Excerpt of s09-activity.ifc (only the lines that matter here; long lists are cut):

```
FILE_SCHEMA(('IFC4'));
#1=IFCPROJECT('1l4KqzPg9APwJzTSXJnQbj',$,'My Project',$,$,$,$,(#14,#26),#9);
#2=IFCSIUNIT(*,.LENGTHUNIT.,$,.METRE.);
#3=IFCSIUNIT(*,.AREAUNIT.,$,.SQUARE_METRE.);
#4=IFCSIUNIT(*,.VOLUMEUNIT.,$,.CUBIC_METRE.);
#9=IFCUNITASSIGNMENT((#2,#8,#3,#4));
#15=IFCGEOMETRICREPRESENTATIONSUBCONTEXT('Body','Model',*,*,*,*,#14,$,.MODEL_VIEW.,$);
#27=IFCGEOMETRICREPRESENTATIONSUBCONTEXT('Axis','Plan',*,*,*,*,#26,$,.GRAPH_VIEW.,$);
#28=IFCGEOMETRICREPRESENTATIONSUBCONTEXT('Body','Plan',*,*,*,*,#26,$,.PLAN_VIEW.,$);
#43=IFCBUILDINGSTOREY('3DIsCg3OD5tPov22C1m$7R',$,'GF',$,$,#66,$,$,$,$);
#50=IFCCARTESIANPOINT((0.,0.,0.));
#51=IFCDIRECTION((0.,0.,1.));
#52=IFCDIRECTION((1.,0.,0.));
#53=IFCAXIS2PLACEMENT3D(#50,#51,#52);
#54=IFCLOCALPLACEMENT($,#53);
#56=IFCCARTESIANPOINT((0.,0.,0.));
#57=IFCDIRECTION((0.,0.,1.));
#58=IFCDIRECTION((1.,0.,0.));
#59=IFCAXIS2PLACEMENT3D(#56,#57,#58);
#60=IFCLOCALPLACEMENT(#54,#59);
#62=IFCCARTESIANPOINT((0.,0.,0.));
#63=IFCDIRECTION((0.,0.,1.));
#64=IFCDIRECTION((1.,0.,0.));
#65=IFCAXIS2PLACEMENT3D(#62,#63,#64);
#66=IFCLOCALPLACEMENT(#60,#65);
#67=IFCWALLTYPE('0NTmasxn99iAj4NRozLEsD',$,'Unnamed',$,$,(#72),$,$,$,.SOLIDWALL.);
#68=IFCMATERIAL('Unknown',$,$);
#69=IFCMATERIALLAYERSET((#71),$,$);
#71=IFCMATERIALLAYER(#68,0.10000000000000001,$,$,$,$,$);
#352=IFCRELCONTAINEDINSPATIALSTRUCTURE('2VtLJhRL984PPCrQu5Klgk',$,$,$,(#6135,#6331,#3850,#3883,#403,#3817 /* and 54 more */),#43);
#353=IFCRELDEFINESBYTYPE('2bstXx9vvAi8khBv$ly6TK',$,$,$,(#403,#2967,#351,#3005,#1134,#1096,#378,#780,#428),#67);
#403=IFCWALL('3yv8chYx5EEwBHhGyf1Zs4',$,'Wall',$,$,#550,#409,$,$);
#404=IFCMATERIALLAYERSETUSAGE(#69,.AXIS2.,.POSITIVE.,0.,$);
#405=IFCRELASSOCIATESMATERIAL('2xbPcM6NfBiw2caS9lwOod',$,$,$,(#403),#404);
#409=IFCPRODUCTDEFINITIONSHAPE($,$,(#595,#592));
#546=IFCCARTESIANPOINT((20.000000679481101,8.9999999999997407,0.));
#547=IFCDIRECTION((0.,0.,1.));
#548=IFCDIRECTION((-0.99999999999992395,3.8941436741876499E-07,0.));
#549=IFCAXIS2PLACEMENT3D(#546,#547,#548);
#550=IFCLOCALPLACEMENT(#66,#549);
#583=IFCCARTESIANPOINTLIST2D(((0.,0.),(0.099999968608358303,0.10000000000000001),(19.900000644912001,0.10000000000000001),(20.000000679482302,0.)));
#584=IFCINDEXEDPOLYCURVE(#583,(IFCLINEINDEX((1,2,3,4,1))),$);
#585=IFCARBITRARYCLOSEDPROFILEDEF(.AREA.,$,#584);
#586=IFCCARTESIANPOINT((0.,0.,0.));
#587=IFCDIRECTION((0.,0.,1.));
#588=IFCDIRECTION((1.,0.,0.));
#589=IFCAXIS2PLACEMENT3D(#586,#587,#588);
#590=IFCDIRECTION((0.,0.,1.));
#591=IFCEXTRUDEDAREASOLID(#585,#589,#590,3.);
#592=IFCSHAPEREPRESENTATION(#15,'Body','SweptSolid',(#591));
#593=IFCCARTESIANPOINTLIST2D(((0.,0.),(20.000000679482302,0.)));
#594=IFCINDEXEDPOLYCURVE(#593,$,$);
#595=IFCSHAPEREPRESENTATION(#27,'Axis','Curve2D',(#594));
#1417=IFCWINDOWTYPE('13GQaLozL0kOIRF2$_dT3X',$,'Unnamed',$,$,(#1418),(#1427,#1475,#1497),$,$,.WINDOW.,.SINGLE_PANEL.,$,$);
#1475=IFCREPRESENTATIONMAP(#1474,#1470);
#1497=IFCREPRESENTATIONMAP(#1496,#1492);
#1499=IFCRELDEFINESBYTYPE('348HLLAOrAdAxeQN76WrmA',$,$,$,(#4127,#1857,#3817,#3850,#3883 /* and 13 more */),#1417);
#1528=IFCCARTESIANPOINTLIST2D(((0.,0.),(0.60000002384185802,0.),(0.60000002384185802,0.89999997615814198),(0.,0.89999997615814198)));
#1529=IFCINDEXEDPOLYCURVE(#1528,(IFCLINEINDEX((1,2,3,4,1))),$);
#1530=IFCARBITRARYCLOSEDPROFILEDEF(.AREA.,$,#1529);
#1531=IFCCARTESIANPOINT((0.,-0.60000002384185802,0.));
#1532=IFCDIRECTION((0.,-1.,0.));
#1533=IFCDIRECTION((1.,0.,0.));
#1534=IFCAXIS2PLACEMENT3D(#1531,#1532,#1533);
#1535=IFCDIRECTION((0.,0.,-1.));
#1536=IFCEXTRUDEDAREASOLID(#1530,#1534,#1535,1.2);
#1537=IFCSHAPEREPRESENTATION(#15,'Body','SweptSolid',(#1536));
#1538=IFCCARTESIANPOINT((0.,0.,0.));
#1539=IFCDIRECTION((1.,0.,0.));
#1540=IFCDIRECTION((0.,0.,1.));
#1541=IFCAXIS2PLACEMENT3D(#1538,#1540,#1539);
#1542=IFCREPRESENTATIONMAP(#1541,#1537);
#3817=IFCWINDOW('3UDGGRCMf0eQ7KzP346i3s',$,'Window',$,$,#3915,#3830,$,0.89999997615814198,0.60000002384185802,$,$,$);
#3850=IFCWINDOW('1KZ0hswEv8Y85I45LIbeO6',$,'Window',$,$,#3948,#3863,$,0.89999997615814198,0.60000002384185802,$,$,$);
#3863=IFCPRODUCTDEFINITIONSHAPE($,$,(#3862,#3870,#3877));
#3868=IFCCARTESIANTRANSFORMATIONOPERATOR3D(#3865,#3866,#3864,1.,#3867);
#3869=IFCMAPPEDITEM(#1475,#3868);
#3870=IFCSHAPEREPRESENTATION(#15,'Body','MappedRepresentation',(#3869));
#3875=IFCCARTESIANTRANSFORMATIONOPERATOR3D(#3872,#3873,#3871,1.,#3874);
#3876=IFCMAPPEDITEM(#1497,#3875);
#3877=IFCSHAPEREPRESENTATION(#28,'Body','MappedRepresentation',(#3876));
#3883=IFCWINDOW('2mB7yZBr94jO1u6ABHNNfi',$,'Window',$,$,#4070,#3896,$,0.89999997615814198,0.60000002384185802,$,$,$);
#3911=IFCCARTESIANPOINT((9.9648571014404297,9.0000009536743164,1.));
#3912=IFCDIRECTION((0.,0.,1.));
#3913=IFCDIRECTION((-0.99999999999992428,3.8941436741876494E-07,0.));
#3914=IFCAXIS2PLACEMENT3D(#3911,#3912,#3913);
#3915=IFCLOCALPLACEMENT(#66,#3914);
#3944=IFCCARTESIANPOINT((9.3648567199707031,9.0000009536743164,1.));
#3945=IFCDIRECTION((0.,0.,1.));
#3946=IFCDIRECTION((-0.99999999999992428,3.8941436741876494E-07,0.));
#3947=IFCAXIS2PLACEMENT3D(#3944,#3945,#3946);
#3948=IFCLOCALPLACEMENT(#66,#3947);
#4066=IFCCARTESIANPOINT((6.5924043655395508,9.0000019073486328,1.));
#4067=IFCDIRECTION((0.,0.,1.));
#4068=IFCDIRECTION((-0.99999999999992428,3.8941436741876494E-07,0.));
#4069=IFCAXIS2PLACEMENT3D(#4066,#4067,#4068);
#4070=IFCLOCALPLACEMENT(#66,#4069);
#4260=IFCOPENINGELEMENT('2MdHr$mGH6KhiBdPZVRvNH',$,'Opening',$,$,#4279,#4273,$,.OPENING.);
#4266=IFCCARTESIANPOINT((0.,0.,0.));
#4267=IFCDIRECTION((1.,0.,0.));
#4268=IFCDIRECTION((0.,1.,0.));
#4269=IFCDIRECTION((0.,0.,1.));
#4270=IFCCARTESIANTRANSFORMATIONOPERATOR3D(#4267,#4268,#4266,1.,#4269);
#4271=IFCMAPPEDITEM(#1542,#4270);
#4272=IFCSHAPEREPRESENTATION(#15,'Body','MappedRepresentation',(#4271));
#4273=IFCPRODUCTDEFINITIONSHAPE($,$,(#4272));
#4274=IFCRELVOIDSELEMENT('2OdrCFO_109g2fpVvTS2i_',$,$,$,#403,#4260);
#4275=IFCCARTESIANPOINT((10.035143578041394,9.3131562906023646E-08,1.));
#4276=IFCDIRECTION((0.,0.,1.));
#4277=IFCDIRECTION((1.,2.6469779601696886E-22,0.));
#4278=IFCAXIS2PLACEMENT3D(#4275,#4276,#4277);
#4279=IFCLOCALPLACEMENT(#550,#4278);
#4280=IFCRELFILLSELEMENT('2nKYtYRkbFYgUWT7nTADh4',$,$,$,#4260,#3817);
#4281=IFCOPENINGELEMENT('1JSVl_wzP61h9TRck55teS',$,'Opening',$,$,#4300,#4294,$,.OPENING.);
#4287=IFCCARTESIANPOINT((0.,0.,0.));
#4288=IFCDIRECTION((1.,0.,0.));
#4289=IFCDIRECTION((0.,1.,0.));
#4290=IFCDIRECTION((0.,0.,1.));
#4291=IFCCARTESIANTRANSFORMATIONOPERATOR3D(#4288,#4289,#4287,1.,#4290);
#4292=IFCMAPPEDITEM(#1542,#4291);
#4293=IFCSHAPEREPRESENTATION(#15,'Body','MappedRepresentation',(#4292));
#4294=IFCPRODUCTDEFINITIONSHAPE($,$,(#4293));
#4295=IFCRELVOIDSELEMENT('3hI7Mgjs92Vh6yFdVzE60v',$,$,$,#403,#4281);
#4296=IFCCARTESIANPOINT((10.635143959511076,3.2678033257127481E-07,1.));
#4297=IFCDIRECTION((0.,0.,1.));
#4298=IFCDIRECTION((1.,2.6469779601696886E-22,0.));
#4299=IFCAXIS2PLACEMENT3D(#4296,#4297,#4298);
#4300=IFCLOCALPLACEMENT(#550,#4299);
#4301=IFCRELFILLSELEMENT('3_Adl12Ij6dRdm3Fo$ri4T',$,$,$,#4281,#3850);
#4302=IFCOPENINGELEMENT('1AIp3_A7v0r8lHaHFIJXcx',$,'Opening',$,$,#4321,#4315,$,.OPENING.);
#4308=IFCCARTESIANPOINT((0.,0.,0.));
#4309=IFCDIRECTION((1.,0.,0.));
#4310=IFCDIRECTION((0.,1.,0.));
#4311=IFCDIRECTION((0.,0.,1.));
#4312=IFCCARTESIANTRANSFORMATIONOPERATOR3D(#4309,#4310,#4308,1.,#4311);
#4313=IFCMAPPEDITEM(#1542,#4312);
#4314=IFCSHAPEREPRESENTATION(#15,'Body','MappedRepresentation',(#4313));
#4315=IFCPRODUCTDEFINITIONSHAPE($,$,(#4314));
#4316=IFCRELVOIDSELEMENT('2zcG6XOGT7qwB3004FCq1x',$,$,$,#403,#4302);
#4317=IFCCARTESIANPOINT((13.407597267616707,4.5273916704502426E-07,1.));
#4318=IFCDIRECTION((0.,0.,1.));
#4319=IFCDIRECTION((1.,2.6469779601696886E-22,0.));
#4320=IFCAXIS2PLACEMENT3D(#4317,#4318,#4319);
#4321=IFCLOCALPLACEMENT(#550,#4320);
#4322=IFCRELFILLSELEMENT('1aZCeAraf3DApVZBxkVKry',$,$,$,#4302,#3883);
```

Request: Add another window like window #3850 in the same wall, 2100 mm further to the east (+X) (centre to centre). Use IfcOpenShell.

```python
import ifcopenshell
import ifcopenshell.api.feature
import ifcopenshell.api.geometry
import ifcopenshell.api.root
import ifcopenshell.geom
import ifcopenshell.util.element
import ifcopenshell.util.placement
import ifcopenshell.util.shape

model = ifcopenshell.open("s09-activity.ifc")
settings = ifcopenshell.geom.settings()


def volume(element):
    """Net volume in cubic metres, openings subtracted."""
    shape = ifcopenshell.geom.create_shape(settings, element)
    return ifcopenshell.util.shape.get_volume(shape.geometry)


window = model.by_guid("1KZ0hswEv8Y85I45LIbeO6")
opening = window.FillsVoids[0].RelatingOpeningElement
wall = opening.VoidsElements[0].RelatingBuildingElement
before = volume(wall)
shift = ifcopenshell.util.placement.get_local_placement(wall.ObjectPlacement)[:3, 0] * -2.1

# copy_class copies the void relationship, type, container and properties, but no geometry.
new_opening = ifcopenshell.api.root.copy_class(model, product=opening)
new_opening.Representation = ifcopenshell.util.element.copy_deep(
    model, opening.Representation, exclude=["IfcGeometricRepresentationContext", "IfcRepresentationMap"]
)
new_window = ifcopenshell.api.root.copy_class(model, product=window)
new_window.Representation = ifcopenshell.util.element.copy_deep(
    model, window.Representation, exclude=["IfcGeometricRepresentationContext", "IfcRepresentationMap"]
)
ifcopenshell.api.feature.add_filling(model, opening=new_opening, element=new_window)

for old, new in ((opening, new_opening), (window, new_window)):
    matrix = ifcopenshell.util.placement.get_local_placement(old.ObjectPlacement)
    matrix[:3, 3] += shift
    ifcopenshell.api.geometry.edit_object_placement(model, product=new, matrix=matrix, is_si=False)

after = volume(wall)

print(f"wall volume {before:.3f} -> {after:.3f} m3")

model.write("s09-activity_edited.ifc")
```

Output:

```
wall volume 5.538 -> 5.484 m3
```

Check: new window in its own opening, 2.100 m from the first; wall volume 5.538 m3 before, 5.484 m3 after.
